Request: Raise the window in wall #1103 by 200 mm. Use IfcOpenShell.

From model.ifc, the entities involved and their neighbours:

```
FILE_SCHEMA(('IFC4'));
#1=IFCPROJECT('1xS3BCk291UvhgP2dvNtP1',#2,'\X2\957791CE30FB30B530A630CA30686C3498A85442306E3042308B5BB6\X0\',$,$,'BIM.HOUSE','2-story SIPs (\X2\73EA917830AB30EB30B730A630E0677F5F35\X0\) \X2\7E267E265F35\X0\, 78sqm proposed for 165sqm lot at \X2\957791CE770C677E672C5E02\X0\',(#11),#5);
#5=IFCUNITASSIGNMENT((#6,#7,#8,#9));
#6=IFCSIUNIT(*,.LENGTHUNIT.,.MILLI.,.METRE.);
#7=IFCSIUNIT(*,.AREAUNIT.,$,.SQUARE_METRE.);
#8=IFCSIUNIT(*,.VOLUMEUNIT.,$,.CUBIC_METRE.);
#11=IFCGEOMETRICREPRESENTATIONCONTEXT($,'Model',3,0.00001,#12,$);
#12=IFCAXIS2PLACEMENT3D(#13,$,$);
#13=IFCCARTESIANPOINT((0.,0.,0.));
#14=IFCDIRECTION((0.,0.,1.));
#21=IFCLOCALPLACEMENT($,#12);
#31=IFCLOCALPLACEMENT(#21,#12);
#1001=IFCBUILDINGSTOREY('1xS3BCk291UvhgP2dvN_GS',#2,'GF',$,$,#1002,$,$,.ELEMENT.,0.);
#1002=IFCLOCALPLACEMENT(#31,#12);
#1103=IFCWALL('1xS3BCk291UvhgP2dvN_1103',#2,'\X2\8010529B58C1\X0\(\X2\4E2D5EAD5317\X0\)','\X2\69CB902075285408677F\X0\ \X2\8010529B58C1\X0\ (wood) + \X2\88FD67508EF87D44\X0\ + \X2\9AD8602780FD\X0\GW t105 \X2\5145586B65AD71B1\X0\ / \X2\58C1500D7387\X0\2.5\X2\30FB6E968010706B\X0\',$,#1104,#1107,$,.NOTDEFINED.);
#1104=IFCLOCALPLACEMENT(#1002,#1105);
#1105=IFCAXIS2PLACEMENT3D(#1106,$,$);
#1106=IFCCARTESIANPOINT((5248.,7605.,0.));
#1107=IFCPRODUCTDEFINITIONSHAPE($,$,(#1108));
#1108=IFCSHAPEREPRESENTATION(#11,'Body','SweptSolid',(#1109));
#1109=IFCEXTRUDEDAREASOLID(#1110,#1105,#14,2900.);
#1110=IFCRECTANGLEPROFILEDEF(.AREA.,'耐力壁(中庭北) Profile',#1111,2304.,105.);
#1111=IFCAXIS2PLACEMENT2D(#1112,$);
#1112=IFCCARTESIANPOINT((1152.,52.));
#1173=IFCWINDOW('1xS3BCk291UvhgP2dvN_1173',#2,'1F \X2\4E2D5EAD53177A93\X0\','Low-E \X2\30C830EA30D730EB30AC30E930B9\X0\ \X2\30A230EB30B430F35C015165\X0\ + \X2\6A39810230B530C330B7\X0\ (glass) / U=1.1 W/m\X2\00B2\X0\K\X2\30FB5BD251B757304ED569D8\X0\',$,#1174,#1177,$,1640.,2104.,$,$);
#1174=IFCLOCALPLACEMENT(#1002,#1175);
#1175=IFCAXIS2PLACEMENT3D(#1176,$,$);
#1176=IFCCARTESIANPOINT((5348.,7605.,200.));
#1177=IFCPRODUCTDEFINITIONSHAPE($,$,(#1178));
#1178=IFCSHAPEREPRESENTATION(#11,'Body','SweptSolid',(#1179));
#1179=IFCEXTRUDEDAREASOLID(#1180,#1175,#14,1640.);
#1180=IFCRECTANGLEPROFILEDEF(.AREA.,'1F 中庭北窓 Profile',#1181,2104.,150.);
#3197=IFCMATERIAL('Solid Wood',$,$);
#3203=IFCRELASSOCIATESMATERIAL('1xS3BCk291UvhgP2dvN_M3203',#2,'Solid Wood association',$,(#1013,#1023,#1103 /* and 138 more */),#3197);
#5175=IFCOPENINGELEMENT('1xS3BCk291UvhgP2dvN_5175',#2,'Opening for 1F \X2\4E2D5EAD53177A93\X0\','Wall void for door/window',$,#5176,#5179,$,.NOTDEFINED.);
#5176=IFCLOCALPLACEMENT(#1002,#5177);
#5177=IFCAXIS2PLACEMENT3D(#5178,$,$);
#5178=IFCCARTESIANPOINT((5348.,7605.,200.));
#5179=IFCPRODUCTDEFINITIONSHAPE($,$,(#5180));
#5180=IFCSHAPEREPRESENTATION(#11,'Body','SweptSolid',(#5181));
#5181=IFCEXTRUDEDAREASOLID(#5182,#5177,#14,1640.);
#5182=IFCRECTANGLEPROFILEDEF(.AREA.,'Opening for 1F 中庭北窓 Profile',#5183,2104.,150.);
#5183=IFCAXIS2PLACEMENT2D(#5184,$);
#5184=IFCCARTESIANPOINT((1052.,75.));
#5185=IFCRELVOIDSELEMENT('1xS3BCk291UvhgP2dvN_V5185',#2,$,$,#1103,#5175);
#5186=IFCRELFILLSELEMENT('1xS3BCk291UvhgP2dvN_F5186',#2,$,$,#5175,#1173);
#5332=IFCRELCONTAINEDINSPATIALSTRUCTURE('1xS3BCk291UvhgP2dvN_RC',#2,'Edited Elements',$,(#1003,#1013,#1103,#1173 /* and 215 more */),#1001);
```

```python
import numpy as np
import ifcopenshell
import ifcopenshell.api.geometry
import ifcopenshell.util.placement
import ifcopenshell.util.unit

model = ifcopenshell.open("model.ifc")
unit_scale = ifcopenshell.util.unit.calculate_unit_scale(model)

window = model.by_guid("1xS3BCk291UvhgP2dvN_1173")
opening = window.FillsVoids[0].RelatingOpeningElement
dz = 0.2 / unit_scale

shift = np.array([0.0, 0.0, dz])
# The window is not placed relative to its opening, so move both.
for product in (opening, window):
    matrix = ifcopenshell.util.placement.get_local_placement(product.ObjectPlacement)
    matrix[:3, 3] += shift
    ifcopenshell.api.geometry.edit_object_placement(model, product=product, matrix=matrix, is_si=False)

print(f"moved by {dz * unit_scale:+.3f} m")

model.write("model_edited.ifc")
```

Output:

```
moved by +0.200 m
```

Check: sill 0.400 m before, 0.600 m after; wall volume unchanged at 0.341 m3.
